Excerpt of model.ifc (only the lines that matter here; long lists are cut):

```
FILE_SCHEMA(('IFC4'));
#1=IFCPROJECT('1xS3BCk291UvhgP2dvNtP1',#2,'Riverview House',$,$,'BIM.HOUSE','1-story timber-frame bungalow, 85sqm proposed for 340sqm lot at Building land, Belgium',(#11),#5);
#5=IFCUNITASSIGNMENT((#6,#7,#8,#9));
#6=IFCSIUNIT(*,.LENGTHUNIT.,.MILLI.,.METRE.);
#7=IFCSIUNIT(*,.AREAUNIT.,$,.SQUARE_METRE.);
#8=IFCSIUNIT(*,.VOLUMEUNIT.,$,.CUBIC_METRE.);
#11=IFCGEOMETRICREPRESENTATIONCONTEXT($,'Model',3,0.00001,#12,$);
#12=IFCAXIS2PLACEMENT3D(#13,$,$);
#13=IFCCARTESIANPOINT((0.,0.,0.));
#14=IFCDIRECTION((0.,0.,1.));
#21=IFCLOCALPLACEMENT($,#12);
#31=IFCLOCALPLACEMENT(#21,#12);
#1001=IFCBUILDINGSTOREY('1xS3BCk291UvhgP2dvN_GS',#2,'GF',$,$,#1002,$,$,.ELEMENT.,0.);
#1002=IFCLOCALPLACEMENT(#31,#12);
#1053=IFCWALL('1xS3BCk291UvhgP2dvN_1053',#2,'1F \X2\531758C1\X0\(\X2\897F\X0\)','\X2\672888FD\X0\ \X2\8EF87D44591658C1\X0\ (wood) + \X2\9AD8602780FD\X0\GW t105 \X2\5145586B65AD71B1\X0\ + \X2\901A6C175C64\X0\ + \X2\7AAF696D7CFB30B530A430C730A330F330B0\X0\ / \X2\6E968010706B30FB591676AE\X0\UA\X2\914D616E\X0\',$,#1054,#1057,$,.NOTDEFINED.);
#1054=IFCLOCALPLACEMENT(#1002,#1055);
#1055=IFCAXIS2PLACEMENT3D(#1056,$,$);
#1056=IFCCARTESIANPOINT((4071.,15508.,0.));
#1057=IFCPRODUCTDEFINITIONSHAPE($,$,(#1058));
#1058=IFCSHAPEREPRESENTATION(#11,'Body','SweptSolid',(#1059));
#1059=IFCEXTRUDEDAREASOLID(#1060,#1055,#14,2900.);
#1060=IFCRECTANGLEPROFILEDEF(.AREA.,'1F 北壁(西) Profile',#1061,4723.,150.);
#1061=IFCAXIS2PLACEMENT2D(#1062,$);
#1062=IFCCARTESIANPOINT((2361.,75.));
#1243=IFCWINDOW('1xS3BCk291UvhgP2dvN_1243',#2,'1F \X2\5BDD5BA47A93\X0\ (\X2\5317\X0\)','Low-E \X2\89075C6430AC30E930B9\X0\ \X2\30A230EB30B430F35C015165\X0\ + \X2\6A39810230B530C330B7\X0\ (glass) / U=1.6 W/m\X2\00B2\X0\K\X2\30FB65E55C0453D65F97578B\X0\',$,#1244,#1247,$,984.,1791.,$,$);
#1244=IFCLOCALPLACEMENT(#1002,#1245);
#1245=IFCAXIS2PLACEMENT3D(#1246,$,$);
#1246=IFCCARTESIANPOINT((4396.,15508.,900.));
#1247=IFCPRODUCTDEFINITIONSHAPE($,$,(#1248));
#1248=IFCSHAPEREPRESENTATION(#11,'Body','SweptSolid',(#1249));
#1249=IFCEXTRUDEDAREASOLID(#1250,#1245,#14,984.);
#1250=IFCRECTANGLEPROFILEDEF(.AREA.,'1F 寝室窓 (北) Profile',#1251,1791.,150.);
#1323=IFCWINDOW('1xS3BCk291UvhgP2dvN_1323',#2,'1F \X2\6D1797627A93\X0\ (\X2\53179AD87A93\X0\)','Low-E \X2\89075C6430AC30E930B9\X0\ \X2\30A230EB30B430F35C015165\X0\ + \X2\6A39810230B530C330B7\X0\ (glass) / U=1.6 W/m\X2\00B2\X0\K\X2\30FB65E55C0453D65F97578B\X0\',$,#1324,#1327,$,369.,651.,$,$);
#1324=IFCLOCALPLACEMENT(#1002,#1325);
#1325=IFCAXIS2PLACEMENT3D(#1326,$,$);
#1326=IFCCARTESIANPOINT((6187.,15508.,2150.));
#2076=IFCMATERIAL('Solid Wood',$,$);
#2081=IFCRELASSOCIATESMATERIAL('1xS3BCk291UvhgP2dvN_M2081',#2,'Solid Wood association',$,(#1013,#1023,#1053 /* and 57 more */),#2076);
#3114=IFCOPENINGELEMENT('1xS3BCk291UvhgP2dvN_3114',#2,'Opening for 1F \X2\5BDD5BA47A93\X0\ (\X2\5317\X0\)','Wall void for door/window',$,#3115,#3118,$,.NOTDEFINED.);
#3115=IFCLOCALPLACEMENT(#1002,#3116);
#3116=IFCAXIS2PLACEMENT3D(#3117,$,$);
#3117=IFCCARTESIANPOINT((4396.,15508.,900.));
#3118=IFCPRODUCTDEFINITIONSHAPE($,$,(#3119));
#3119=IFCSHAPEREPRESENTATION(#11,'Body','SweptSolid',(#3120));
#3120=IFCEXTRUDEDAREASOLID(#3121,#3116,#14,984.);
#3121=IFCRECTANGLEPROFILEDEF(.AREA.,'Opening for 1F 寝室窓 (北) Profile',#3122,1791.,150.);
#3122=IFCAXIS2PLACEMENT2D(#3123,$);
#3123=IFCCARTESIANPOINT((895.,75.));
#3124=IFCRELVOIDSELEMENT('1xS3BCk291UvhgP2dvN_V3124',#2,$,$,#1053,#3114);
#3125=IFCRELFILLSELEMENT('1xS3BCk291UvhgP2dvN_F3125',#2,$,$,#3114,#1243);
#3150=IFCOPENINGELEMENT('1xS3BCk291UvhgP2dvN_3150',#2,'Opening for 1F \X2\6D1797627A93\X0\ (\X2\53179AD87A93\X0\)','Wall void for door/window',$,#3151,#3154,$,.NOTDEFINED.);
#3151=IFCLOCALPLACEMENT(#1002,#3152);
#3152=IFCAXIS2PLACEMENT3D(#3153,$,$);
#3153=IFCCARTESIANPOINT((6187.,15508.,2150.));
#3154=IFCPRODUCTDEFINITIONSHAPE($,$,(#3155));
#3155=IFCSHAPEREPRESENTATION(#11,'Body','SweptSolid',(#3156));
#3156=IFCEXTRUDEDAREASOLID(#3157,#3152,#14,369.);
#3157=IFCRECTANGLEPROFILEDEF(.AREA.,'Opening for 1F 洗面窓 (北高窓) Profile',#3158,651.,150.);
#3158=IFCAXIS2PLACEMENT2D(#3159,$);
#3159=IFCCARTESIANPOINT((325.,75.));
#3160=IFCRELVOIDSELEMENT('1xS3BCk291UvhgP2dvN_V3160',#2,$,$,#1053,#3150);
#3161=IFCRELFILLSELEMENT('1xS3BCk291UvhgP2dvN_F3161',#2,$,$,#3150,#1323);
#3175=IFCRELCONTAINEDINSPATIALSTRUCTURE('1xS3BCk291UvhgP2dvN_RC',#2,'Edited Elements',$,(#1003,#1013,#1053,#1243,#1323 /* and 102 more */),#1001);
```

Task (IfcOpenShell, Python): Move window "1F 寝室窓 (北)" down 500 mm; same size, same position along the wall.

```python
import numpy as np
import ifcopenshell
import ifcopenshell.api.geometry
import ifcopenshell.util.placement
import ifcopenshell.util.unit

model = ifcopenshell.open("model.ifc")
unit_scale = ifcopenshell.util.unit.calculate_unit_scale(model)

window = model.by_id(1243)
opening = window.FillsVoids[0].RelatingOpeningElement
dz = -0.5 / unit_scale

shift = np.array([0.0, 0.0, dz])
# The window is not placed relative to its opening, so move both.
for product in (opening, window):
    matrix = ifcopenshell.util.placement.get_local_placement(product.ObjectPlacement)
    matrix[:3, 3] += shift
    ifcopenshell.api.geometry.edit_object_placement(model, product=product, matrix=matrix, is_si=False)

print(f"moved by {dz * unit_scale:+.3f} m")

model.write("model_rev.ifc")
```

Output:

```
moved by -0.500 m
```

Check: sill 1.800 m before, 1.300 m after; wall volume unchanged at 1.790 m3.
